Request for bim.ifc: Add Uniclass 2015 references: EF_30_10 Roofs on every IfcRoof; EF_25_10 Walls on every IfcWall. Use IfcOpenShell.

First a look at what the model holds.

```python
import ifcopenshell

model = ifcopenshell.open("bim.ifc")
print(model.schema)
print("classifications:", [c.Name for c in model.by_type("IfcClassification")])
for ifc_class in ("IfcDoor", "IfcRoof", "IfcStair", "IfcWall", "IfcWindow"):
    print(ifc_class, len(model.by_type(ifc_class)))
```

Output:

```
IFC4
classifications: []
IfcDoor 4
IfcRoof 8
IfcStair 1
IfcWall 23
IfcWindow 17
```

```python
import ifcopenshell
import ifcopenshell.api.classification

model = ifcopenshell.open("bim.ifc")

system = ifcopenshell.api.classification.add_classification(model, classification="Uniclass 2015")

codes = {
    "IfcRoof": ("EF_30_10", "Roofs"),
    "IfcWall": ("EF_25_10", "Walls"),
}
for ifc_class, (code, name) in codes.items():
    products = model.by_type(ifc_class)
    ifcopenshell.api.classification.add_reference(
        model, products=products, classification=system, identification=code, name=name
    )
    print(code, len(products))

model.write("bim_edited.ifc")
```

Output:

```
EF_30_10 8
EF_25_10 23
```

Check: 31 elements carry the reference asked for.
